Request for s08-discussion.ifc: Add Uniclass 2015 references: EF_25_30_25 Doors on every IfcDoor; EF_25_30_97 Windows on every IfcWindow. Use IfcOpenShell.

First a look at what the model holds.

```python
import ifcopenshell

model = ifcopenshell.open("s08-discussion.ifc")
print(model.schema)
print("classifications:", [c.Name for c in model.by_type("IfcClassification")])
for ifc_class in ("IfcDoor", "IfcRoof", "IfcStair", "IfcWall", "IfcWindow"):
    print(ifc_class, len(model.by_type(ifc_class)))
```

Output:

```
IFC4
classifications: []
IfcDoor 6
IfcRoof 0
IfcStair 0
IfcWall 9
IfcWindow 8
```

```python
import ifcopenshell
import ifcopenshell.api.classification

model = ifcopenshell.open("s08-discussion.ifc")

system = ifcopenshell.api.classification.add_classification(model, classification="Uniclass 2015")

codes = {
    "IfcDoor": ("EF_25_30_25", "Doors"),
    "IfcWindow": ("EF_25_30_97", "Windows"),
}
for ifc_class, (code, name) in codes.items():
    products = model.by_type(ifc_class)
    ifcopenshell.api.classification.add_reference(
        model, products=products, classification=system, identification=code, name=name
    )
    print(code, len(products))

model.write("s08-discussion_v2.ifc")
```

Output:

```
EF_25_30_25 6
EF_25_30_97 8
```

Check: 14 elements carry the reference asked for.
